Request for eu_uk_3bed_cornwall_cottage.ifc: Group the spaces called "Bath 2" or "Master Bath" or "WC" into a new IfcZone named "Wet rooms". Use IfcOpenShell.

First a look at what the model holds.

```python
import ifcopenshell

model = ifcopenshell.open("eu_uk_3bed_cornwall_cottage.ifc")
print(model.schema)
seen = {}
for space in model.by_type("IfcSpace"):
    seen[space.LongName] = seen.get(space.LongName, 0) + 1
for name, count in sorted(seen.items(), key=str):
    print(count, "x", name)
print("zones:", [z.Name for z in model.by_type("IfcZone")][:20])
```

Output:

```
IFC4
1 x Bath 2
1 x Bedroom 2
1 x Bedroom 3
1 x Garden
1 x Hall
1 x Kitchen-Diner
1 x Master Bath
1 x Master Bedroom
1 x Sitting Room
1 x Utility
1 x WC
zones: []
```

```python
import ifcopenshell
import ifcopenshell.api.group
import ifcopenshell.api.root

model = ifcopenshell.open("eu_uk_3bed_cornwall_cottage.ifc")

names = {"Bath 2", "Master Bath", "WC"}
spaces = [s for s in model.by_type("IfcSpace") if s.LongName in names]

zone = ifcopenshell.api.root.create_entity(model, ifc_class="IfcZone", name="Wet rooms")
ifcopenshell.api.group.assign_group(model, products=spaces, group=zone)
print(len(spaces), "spaces in", zone.Name)

model.write("eu_uk_3bed_cornwall_cottage_updated.ifc")
```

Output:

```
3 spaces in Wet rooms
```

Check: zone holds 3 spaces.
